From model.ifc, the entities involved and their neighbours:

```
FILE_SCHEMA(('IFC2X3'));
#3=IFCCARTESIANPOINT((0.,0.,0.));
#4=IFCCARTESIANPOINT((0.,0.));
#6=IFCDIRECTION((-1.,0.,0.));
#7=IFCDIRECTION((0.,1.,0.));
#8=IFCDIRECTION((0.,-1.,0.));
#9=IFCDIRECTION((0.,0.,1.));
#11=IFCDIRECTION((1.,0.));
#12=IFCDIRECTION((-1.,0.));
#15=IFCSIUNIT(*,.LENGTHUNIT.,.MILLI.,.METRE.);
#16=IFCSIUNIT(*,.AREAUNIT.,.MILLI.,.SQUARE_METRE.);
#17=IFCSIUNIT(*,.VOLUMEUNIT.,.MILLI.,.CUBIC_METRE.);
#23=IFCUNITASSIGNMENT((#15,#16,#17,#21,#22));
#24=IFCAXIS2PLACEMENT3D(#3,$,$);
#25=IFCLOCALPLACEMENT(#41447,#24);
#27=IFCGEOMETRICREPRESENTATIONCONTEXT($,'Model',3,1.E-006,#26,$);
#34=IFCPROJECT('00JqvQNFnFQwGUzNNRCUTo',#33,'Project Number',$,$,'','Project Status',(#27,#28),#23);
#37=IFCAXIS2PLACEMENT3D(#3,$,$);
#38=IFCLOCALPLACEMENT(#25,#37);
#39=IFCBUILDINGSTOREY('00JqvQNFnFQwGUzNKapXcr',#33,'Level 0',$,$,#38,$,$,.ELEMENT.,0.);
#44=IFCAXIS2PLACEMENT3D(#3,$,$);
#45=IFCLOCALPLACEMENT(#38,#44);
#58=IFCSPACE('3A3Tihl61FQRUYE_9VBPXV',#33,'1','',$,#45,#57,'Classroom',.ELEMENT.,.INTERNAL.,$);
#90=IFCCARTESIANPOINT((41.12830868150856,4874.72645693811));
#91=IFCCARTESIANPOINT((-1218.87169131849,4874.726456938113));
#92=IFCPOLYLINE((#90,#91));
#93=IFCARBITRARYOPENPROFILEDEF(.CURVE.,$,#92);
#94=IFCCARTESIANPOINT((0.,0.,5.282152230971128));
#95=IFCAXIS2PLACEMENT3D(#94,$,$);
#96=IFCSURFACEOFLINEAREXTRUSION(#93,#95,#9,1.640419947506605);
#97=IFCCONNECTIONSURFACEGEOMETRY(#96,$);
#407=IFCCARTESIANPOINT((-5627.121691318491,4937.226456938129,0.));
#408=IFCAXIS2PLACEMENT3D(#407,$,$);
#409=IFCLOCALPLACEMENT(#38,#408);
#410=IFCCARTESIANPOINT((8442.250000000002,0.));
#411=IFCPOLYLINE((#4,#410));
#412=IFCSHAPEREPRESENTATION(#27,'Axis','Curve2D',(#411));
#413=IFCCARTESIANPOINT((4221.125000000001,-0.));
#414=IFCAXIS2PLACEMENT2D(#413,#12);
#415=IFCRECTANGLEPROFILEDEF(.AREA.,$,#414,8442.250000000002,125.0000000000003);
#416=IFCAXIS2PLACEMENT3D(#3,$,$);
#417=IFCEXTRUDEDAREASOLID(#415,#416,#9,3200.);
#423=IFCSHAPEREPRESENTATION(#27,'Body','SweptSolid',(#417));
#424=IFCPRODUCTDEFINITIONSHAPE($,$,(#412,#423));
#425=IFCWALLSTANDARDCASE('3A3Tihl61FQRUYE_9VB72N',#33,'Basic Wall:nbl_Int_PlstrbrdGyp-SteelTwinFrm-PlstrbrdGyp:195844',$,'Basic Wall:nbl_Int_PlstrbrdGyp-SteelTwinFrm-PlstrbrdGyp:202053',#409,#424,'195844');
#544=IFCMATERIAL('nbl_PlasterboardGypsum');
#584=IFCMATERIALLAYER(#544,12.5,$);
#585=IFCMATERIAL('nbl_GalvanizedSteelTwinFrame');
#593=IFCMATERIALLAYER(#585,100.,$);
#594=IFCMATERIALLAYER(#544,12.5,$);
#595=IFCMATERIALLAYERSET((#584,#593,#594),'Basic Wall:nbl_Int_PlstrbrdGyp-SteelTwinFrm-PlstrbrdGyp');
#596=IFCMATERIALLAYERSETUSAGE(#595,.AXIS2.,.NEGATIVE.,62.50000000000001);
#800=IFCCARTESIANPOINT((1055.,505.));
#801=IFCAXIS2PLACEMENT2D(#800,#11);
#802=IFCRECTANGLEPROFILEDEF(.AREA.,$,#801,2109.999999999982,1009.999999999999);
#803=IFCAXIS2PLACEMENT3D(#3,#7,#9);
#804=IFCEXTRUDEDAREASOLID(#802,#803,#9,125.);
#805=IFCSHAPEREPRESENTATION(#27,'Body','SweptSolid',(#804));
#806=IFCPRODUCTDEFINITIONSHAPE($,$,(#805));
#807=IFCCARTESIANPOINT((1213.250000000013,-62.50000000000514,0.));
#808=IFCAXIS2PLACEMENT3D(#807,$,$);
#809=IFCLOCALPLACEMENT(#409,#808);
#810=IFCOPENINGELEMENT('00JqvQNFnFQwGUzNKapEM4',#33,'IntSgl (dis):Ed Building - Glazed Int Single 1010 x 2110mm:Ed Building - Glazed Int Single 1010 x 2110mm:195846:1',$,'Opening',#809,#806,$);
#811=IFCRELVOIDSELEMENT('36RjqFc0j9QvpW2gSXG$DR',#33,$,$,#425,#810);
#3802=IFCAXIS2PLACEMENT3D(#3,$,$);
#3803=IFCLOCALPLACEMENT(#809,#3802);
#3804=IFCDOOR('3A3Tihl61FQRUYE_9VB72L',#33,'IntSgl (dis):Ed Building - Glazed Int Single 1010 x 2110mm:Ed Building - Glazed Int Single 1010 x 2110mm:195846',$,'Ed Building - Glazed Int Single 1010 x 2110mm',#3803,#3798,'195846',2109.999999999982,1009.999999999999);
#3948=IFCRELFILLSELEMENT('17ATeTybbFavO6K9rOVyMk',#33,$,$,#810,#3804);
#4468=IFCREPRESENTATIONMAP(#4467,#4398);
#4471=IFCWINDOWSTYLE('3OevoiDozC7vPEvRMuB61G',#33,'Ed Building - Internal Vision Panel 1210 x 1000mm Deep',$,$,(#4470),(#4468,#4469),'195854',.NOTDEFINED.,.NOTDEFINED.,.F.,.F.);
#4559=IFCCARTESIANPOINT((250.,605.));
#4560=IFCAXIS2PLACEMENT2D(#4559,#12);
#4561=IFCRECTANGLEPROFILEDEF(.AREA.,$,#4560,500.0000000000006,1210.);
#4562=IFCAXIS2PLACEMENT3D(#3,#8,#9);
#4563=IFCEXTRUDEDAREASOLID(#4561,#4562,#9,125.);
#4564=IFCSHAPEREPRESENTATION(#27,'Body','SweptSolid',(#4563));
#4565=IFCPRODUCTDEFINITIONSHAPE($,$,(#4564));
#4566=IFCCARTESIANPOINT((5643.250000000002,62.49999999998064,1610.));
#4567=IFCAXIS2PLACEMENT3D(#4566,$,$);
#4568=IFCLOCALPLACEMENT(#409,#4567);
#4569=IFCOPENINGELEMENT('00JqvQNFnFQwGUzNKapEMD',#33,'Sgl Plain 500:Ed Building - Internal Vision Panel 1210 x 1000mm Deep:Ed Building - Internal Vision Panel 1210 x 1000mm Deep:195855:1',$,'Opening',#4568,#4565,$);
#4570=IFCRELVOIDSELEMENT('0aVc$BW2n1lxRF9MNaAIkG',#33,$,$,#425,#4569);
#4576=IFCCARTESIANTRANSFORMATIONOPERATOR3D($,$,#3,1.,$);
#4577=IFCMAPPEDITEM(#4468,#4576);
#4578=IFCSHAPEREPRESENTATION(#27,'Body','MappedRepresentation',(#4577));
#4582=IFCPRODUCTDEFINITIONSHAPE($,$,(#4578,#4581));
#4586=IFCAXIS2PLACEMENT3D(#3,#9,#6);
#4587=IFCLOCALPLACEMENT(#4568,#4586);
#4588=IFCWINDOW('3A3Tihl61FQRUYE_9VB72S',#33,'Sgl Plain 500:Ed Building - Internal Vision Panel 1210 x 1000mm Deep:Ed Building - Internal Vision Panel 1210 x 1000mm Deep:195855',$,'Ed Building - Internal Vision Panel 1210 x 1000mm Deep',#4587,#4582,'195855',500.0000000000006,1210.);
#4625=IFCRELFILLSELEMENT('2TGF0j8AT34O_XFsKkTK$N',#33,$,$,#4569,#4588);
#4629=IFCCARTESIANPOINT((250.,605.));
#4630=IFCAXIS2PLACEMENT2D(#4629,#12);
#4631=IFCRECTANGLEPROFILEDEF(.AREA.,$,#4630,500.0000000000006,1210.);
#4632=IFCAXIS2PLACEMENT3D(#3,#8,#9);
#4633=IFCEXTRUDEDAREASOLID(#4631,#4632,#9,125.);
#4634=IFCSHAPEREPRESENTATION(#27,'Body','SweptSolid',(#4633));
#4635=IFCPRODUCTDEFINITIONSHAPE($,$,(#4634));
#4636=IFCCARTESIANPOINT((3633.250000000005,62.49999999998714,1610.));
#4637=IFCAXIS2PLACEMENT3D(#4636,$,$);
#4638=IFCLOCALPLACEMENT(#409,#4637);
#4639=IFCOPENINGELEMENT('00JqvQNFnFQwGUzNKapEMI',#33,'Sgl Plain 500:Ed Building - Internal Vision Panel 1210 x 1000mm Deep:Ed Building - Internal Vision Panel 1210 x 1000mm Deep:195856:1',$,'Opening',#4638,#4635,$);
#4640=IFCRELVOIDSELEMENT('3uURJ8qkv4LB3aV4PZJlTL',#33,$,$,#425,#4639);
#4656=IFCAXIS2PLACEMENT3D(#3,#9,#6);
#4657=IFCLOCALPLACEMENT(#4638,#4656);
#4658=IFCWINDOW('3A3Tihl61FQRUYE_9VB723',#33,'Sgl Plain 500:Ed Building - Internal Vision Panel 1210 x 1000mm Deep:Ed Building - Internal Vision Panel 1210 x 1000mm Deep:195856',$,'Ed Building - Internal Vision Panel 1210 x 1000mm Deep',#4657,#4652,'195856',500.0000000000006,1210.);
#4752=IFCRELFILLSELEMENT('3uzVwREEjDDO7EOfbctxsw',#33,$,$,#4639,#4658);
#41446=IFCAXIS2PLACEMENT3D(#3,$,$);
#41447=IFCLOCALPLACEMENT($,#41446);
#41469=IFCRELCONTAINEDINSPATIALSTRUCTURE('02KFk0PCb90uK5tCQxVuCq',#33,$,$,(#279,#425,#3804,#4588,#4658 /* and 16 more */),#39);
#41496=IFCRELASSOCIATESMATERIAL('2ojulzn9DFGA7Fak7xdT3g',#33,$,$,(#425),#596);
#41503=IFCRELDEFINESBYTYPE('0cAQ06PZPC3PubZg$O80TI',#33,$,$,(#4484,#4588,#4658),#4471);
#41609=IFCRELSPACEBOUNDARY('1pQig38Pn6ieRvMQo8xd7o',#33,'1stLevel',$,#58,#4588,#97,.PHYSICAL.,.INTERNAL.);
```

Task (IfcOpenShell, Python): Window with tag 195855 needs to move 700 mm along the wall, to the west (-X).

```python
import numpy as np
import ifcopenshell
import ifcopenshell.api.geometry
import ifcopenshell.util.placement
import ifcopenshell.util.unit

model = ifcopenshell.open("model.ifc")
unit_scale = ifcopenshell.util.unit.calculate_unit_scale(model)

window = model.by_guid("3A3Tihl61FQRUYE_9VB72S")
opening = window.FillsVoids[0].RelatingOpeningElement
wall = opening.VoidsElements[0].RelatingBuildingElement

wall_matrix = ifcopenshell.util.placement.get_local_placement(wall.ObjectPlacement)
shift = wall_matrix[:3, 0] * -0.7 / unit_scale
before = ifcopenshell.util.placement.get_local_placement(window.ObjectPlacement)[:3, 3].copy()

# The window is placed relative to its opening, so it follows when the opening moves.
matrix = ifcopenshell.util.placement.get_local_placement(opening.ObjectPlacement)
matrix[:3, 3] += shift
ifcopenshell.api.geometry.edit_object_placement(
    model, product=opening, matrix=matrix, is_si=False, should_transform_children=True
)

# Space boundary surfaces are stored in each space's coordinates; move them too.
for rel in window.ProvidesBoundaries:
    if not rel.ConnectionGeometry:
        continue
    surface = rel.ConnectionGeometry.SurfaceOnRelatingElement
    space_matrix = ifcopenshell.util.placement.get_local_placement(rel.RelatingSpace.ObjectPlacement)
    point = np.array(surface.Position.Location.Coordinates) + space_matrix[:3, :3].T @ shift
    surface.Position = model.createIfcAxis2Placement3D(
        model.createIfcCartesianPoint(point.tolist()), surface.Position.Axis, surface.Position.RefDirection
    )

after = ifcopenshell.util.placement.get_local_placement(window.ObjectPlacement)[:3, 3]
print("window moved by", (after - before).round(3) + 0.0)

model.write("model-out.ifc")
```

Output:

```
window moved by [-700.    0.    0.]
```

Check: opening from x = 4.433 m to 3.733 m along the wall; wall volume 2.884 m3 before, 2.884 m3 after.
